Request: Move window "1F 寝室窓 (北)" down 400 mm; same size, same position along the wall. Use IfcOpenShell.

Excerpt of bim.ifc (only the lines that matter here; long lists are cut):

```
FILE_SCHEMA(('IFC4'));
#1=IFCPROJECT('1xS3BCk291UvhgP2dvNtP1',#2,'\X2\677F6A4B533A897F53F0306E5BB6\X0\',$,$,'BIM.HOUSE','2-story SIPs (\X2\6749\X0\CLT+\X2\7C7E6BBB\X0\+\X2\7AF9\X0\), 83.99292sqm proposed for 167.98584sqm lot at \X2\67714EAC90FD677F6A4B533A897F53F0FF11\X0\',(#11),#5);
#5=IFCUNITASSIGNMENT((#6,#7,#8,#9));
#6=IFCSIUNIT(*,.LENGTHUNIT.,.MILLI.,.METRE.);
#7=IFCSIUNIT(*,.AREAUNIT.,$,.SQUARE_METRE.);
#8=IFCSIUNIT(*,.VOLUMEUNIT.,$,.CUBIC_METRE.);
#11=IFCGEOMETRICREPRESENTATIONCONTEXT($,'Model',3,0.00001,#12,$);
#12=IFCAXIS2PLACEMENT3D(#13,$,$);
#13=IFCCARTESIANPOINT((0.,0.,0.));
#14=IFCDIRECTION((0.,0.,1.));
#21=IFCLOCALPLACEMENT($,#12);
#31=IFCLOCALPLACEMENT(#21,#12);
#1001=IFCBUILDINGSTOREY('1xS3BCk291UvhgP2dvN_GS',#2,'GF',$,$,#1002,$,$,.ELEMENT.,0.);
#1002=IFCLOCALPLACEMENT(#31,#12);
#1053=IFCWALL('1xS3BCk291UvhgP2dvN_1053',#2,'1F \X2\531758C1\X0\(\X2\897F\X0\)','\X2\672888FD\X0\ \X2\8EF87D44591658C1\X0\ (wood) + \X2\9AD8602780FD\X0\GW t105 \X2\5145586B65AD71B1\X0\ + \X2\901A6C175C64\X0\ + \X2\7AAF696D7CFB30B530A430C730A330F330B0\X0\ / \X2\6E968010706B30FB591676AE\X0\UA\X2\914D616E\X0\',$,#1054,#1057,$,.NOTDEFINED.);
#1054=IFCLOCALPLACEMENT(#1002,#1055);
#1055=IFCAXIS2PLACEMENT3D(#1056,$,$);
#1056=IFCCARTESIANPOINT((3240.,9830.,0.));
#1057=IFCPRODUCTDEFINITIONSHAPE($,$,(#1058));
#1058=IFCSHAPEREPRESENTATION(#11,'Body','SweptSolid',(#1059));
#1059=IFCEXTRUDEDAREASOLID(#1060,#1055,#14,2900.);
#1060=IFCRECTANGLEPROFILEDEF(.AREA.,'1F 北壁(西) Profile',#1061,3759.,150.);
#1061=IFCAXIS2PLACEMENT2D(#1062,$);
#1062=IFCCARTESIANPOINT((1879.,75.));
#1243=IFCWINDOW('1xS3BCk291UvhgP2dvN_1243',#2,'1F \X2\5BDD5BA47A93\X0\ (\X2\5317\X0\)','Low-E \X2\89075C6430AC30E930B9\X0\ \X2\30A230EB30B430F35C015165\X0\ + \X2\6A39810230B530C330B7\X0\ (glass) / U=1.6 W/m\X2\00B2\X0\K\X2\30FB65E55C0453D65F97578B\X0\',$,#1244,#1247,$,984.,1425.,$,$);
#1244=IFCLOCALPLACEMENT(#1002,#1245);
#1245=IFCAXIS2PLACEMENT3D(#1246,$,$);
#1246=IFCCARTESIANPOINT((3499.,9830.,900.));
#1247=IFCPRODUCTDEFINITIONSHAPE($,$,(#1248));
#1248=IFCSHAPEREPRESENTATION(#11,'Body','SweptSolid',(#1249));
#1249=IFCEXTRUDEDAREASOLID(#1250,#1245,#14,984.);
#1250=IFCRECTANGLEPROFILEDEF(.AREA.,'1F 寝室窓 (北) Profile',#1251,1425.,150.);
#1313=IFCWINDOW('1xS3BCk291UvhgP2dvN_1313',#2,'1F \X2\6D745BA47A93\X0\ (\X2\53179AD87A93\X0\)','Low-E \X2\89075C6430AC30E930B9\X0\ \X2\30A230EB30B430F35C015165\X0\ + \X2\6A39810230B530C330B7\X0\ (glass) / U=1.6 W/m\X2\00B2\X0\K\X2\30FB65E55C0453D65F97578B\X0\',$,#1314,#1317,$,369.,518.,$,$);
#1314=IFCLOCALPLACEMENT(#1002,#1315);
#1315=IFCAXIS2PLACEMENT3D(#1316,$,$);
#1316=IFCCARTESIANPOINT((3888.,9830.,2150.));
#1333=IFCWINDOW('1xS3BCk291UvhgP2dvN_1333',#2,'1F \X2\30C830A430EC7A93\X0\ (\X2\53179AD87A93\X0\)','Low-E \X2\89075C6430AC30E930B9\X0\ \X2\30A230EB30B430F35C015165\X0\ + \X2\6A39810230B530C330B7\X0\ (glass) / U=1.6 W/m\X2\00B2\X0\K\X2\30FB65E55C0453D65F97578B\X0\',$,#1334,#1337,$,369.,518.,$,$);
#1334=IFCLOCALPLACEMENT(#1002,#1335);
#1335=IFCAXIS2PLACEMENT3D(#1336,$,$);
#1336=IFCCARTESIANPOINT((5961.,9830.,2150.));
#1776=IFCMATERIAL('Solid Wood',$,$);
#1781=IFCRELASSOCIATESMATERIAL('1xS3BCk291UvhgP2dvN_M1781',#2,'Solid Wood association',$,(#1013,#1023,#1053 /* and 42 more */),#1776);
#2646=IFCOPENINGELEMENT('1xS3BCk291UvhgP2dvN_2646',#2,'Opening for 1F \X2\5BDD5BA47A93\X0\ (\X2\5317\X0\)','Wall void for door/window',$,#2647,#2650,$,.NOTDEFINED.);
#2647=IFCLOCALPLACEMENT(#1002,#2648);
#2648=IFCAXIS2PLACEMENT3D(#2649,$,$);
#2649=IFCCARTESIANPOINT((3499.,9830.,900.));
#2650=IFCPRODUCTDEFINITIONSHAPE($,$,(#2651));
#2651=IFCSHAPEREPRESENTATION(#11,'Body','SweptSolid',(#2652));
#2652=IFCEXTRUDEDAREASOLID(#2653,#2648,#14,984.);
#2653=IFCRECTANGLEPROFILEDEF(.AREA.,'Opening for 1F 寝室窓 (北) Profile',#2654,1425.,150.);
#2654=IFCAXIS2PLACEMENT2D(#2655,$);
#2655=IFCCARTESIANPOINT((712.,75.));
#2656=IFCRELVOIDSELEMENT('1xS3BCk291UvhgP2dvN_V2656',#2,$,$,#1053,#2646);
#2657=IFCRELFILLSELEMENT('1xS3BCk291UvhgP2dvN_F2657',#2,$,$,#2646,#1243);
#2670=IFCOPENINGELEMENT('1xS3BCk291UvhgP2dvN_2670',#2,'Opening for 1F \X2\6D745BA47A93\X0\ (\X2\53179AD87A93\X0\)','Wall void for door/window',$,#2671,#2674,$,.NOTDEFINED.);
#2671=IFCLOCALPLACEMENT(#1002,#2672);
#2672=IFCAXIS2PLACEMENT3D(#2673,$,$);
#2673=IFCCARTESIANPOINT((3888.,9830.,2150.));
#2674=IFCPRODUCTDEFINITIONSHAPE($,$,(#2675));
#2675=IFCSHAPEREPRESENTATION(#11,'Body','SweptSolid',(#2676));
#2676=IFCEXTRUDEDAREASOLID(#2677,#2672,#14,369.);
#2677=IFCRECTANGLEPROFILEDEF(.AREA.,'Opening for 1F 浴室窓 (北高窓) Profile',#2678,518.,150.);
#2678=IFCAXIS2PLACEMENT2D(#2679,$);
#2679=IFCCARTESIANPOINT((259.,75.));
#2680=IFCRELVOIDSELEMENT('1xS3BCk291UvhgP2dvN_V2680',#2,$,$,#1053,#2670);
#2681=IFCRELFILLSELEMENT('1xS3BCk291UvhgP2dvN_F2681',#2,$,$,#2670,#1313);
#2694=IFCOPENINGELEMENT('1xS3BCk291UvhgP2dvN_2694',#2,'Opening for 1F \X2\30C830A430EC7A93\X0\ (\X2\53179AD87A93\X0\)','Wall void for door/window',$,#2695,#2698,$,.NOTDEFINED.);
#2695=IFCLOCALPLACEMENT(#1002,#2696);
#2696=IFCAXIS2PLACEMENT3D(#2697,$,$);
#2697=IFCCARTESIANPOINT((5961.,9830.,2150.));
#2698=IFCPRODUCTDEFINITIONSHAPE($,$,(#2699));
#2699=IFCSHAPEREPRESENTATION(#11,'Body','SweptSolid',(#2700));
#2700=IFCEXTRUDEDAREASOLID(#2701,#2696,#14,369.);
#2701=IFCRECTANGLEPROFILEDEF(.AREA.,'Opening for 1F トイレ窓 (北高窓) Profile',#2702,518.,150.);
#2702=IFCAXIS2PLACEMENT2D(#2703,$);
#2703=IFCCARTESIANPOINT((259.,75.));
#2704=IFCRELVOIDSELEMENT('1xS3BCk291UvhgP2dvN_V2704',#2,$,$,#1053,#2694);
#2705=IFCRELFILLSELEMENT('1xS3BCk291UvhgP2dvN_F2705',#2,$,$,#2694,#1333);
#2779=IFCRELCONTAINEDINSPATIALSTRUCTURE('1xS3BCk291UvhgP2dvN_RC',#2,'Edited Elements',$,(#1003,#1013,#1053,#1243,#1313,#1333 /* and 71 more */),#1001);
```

```python
import numpy as np
import ifcopenshell
import ifcopenshell.api.geometry
import ifcopenshell.util.placement
import ifcopenshell.util.unit

model = ifcopenshell.open("bim.ifc")
unit_scale = ifcopenshell.util.unit.calculate_unit_scale(model)

window = model.by_id(1243)
opening = window.FillsVoids[0].RelatingOpeningElement
dz = -400.0

shift = np.array([0.0, 0.0, dz])
# The window is not placed relative to its opening, so move both.
for product in (opening, window):
    matrix = ifcopenshell.util.placement.get_local_placement(product.ObjectPlacement)
    matrix[:3, 3] += shift
    ifcopenshell.api.geometry.edit_object_placement(model, product=product, matrix=matrix, is_si=False)

print(f"moved by {dz * unit_scale:+.3f} m")

model.write("bim_rev.ifc")
```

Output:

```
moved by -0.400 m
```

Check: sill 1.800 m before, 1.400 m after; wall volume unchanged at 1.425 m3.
